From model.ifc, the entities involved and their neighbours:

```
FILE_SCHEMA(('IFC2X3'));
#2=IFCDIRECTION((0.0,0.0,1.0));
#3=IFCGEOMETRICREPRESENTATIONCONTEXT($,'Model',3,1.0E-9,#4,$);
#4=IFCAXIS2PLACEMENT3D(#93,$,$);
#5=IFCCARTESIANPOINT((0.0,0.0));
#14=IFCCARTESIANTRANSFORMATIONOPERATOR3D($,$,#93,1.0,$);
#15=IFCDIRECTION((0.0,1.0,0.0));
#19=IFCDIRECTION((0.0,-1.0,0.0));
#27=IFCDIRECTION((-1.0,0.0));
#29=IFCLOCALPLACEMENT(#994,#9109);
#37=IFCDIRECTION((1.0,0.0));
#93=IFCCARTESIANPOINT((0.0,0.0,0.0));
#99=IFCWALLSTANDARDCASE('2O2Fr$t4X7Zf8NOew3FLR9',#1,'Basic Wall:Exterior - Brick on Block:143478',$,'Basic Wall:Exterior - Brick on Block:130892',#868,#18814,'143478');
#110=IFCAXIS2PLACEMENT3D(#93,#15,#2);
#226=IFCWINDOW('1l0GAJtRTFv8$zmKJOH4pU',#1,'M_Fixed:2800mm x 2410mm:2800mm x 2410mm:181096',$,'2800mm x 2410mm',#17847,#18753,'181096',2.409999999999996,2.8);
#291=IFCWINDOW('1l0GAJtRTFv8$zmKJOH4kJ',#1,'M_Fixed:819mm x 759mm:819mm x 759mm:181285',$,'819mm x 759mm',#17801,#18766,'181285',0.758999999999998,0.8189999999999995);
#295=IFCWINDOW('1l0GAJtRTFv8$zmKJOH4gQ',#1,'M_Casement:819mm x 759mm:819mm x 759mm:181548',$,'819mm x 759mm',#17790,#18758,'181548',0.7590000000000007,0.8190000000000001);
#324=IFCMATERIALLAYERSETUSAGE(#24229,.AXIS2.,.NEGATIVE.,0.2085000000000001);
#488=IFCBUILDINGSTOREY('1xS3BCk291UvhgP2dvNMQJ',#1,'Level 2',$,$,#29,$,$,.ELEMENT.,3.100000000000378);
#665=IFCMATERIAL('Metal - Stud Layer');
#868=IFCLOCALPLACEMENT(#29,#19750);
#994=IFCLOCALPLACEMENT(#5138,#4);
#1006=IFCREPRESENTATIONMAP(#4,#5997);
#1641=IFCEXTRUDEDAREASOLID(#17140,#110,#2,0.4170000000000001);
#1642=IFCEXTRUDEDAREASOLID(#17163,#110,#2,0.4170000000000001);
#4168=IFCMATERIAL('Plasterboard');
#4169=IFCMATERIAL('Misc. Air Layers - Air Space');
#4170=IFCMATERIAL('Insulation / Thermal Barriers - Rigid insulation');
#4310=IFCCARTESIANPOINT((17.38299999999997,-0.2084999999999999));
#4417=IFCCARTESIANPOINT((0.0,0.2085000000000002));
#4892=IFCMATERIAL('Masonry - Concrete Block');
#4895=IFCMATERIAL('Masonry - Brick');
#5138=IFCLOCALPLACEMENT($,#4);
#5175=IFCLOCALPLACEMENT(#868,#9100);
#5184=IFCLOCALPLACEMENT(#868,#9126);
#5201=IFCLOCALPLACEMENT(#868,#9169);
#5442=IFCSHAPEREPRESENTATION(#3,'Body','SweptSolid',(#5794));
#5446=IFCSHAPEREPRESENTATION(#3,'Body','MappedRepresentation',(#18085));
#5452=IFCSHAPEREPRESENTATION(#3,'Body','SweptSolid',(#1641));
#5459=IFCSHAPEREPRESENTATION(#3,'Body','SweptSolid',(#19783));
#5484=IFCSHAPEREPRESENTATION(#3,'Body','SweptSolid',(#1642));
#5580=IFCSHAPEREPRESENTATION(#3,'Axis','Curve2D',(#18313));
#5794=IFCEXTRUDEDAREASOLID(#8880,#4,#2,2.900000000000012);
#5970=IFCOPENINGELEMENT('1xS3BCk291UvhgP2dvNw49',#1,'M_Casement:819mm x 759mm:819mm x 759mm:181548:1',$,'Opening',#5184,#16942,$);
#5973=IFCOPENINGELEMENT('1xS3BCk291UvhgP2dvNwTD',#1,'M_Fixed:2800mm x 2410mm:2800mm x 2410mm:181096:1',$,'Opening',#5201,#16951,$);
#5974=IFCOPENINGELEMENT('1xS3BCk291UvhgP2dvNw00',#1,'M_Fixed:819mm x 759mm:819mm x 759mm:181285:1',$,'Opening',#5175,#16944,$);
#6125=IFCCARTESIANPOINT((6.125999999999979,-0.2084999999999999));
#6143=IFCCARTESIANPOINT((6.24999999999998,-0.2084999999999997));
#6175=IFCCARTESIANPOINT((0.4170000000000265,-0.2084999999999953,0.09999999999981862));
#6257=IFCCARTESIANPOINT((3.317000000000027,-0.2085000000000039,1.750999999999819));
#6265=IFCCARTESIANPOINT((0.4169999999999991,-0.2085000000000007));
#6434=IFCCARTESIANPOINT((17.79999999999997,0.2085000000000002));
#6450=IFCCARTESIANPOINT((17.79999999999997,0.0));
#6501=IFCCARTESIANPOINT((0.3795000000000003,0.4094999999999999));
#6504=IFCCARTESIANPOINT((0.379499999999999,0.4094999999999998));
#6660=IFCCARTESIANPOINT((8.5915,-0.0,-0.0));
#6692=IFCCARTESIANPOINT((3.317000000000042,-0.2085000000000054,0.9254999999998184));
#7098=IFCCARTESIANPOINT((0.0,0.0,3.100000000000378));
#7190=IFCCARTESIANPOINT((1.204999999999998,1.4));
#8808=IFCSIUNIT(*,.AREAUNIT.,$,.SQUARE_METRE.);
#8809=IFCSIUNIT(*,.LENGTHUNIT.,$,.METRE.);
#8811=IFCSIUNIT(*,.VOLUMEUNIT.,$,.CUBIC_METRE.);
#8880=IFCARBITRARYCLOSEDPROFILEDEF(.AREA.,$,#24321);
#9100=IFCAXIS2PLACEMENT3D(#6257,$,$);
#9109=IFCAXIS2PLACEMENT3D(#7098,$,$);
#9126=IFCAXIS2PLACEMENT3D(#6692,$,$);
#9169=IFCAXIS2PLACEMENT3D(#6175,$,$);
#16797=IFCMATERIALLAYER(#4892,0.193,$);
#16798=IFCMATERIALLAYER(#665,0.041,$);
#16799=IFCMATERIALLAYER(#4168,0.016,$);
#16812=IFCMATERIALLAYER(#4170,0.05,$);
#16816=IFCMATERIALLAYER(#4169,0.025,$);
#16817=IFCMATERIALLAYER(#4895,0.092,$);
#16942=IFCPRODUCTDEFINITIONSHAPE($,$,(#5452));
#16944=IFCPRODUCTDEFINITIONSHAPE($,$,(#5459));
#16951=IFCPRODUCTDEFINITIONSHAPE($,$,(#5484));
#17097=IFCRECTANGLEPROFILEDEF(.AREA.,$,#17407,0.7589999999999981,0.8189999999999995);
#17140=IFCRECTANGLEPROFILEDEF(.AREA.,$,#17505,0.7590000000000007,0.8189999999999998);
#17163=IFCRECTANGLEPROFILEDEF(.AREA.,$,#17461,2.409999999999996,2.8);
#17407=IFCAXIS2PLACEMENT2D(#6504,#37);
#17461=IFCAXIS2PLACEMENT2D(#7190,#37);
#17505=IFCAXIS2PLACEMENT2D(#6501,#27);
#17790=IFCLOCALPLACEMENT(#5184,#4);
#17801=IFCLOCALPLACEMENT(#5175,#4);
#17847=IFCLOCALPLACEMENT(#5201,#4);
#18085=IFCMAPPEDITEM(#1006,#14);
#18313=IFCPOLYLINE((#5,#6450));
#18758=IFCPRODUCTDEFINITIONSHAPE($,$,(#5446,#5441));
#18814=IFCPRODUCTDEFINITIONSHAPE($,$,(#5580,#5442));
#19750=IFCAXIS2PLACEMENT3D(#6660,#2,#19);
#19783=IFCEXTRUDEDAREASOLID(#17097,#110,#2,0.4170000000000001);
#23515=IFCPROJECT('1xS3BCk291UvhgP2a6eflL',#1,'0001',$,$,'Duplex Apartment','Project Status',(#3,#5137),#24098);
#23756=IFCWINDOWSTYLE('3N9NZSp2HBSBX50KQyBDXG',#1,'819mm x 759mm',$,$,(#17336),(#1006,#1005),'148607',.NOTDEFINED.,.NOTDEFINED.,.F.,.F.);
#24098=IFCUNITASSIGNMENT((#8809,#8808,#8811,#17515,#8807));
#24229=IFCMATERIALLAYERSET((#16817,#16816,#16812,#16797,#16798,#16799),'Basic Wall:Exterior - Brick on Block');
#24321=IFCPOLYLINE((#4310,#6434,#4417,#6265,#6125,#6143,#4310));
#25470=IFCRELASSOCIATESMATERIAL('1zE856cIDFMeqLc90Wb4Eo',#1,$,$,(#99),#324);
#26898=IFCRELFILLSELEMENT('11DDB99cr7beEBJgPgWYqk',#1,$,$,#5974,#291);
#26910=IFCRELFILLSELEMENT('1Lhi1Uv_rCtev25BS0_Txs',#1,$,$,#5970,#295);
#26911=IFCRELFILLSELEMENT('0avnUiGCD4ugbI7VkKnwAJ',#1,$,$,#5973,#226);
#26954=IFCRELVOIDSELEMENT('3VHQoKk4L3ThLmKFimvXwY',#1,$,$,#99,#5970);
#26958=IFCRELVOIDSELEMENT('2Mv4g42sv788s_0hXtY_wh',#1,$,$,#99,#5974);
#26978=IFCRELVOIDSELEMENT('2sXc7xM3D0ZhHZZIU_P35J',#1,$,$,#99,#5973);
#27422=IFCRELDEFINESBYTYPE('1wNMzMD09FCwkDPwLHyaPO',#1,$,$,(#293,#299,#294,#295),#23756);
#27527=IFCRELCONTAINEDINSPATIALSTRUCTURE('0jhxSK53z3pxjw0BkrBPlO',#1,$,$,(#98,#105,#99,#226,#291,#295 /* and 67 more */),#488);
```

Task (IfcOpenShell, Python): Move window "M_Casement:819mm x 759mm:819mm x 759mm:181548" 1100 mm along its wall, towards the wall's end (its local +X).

```python
import ifcopenshell
import ifcopenshell.api.geometry
import ifcopenshell.util.placement
import ifcopenshell.util.unit

model = ifcopenshell.open("model.ifc")
unit_scale = ifcopenshell.util.unit.calculate_unit_scale(model)

window = model.by_guid("1l0GAJtRTFv8$zmKJOH4gQ")
opening = window.FillsVoids[0].RelatingOpeningElement
wall = opening.VoidsElements[0].RelatingBuildingElement

wall_matrix = ifcopenshell.util.placement.get_local_placement(wall.ObjectPlacement)
shift = wall_matrix[:3, 0] * 1.1 / unit_scale
before = ifcopenshell.util.placement.get_local_placement(window.ObjectPlacement)[:3, 3].copy()

# The window is placed relative to its opening, so it follows when the opening moves.
matrix = ifcopenshell.util.placement.get_local_placement(opening.ObjectPlacement)
matrix[:3, 3] += shift
ifcopenshell.api.geometry.edit_object_placement(
    model, product=opening, matrix=matrix, is_si=False, should_transform_children=True
)

after = ifcopenshell.util.placement.get_local_placement(window.ObjectPlacement)[:3, 3]
print("window moved by", (after - before).round(3) + 0.0)

model.write("model_updated.ifc")
```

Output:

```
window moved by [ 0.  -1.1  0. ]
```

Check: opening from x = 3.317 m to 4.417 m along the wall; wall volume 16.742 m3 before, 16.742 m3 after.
